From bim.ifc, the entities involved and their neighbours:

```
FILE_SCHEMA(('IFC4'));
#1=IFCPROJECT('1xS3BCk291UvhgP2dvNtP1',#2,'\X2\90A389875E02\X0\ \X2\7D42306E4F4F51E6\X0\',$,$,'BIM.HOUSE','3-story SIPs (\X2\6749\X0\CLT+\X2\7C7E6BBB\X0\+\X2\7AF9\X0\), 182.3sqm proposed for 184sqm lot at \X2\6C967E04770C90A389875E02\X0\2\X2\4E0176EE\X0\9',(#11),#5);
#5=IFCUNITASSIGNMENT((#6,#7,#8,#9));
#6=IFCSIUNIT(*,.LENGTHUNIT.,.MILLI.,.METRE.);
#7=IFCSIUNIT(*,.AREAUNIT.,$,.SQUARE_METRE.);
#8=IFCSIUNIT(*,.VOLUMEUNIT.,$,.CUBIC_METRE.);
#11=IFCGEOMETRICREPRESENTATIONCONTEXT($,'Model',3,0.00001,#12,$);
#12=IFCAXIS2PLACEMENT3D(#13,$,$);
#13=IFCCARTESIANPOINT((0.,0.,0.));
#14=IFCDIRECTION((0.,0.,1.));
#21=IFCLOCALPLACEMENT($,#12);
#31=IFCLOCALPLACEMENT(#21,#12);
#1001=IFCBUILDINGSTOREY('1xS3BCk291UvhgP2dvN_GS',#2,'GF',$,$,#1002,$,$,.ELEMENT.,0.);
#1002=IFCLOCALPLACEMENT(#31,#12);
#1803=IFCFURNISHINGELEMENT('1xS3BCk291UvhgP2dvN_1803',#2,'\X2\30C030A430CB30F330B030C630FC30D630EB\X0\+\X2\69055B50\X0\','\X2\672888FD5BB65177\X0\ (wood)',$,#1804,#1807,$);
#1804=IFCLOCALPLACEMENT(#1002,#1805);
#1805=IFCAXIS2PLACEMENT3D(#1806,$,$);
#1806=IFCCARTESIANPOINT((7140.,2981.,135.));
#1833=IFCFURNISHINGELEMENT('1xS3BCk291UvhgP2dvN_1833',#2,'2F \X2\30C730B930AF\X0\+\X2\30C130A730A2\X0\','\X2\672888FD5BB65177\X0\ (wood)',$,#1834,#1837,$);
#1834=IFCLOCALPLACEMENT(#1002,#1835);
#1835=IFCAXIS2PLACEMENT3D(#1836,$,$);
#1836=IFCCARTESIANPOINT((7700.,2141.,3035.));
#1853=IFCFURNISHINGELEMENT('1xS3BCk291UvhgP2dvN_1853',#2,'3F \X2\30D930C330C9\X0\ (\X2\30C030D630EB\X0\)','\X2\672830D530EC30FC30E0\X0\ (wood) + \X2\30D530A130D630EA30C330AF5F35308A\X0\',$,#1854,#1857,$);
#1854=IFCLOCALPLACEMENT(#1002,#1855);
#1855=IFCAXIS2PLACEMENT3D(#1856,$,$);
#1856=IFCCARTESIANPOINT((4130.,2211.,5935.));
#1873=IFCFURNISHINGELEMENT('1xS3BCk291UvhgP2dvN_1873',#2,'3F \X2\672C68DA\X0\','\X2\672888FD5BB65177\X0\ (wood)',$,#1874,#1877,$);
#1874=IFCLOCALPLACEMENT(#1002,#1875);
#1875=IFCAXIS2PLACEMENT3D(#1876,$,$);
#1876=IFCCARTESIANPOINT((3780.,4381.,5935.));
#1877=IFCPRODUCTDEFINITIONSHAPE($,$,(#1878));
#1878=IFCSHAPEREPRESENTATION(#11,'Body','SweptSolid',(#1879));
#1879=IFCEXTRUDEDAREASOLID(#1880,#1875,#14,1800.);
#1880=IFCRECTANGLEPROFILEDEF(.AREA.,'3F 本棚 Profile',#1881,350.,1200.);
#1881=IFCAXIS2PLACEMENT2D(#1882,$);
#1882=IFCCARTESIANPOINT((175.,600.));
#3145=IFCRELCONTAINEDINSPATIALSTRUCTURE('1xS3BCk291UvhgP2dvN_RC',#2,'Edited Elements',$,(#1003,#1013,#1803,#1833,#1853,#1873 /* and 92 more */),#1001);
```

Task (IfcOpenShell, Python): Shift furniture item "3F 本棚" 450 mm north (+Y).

```python
import ifcopenshell
import ifcopenshell.api.geometry
import ifcopenshell.util.placement
import ifcopenshell.util.unit

model = ifcopenshell.open("bim.ifc")
unit_scale = ifcopenshell.util.unit.calculate_unit_scale(model)

item = model.by_id(1873)
matrix = ifcopenshell.util.placement.get_local_placement(item.ObjectPlacement)
matrix[1, 3] += 0.45 / unit_scale
ifcopenshell.api.geometry.edit_object_placement(model, product=item, matrix=matrix, is_si=False)

print(ifcopenshell.util.placement.get_local_placement(item.ObjectPlacement).round(3) + 0.0)

model.write("bim-out.ifc")
```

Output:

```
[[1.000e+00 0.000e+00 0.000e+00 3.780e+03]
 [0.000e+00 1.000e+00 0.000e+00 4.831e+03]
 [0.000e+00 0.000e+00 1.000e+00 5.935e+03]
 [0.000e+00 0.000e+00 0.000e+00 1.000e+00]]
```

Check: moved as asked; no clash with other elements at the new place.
